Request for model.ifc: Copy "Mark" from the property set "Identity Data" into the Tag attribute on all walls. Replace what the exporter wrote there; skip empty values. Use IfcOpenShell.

First a look at what the model holds.

```python
import ifcopenshell
import ifcopenshell.util.element

model = ifcopenshell.open("model.ifc")
print(model.schema)
walls = model.by_type("IfcWall")
print(len(walls), "walls")
for e in walls[:8]:
    source = ifcopenshell.util.element.get_pset(e, "Identity Data", "Mark")
    target = e.Tag
    print(e.id(), repr(source), repr(target), sep=" | ")
```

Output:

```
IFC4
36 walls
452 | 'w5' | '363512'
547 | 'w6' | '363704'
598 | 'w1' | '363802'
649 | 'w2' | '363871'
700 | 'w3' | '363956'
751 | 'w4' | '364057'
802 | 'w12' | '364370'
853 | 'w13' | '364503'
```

```python
import ifcopenshell
import ifcopenshell.util.element

model = ifcopenshell.open("model.ifc")

count = 0
for e in model.by_type("IfcWall"):
    value = ifcopenshell.util.element.get_pset(e, "Identity Data", "Mark")
    current = e.Tag
    if not value or not value.strip() or current == value:
        continue
    e.Tag = value
    count += 1

print(count, "walls updated")

model.write("model_edited.ifc")
```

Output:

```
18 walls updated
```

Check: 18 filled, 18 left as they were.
